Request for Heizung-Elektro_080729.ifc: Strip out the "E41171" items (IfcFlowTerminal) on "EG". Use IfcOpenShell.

First a look at what the model holds.

```python
import ifcopenshell
import ifcopenshell.util.element

model = ifcopenshell.open("Heizung-Elektro_080729.ifc")
print(model.schema)
storey = next(s for s in model.by_type("IfcBuildingStorey") if s.Name == "EG")
terminals = [e for e in ifcopenshell.util.element.get_decomposition(storey) if e.is_a("IfcFlowTerminal")]
seen = {}
for e in terminals:
    element_type = ifcopenshell.util.element.get_type(e)
    name = element_type.Name if element_type not in (None, e) else None
    seen[name] = seen.get(name, 0) + 1
for name, count in sorted(seen.items(), key=str):
    print(count, "x", name)
```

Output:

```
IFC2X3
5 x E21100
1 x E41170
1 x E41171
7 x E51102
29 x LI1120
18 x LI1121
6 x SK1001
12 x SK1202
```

```python
import ifcopenshell
import ifcopenshell.api.root
import ifcopenshell.util.element

model = ifcopenshell.open("Heizung-Elektro_080729.ifc")

storey = next(s for s in model.by_type("IfcBuildingStorey") if s.Name == "EG")
terminals = [e for e in ifcopenshell.util.element.get_decomposition(storey) if e.is_a("IfcFlowTerminal")]
targets = [e for e in terminals if (t := ifcopenshell.util.element.get_type(e)) not in (None, e) and t.Name == "E41171"]

for e in targets:
    ifcopenshell.api.root.remove_product(model, product=e)
print(len(targets), "removed")

model.write("Heizung-Elektro_080729_updated.ifc")
```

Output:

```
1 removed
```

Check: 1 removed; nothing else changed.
